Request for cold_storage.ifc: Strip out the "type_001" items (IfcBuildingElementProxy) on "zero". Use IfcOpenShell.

First a look at what the model holds.

```python
import ifcopenshell
import ifcopenshell.util.element

model = ifcopenshell.open("cold_storage.ifc")
print(model.schema)
storey = next(s for s in model.by_type("IfcBuildingStorey") if s.Name == "zero")
proxies = [e for e in ifcopenshell.util.element.get_decomposition(storey) if e.is_a("IfcBuildingElementProxy")]
seen = {}
for e in proxies:
    element_type = ifcopenshell.util.element.get_type(e)
    name = element_type.Name if element_type not in (None, e) else None
    seen[name] = seen.get(name, 0) + 1
for name, count in sorted(seen.items(), key=str):
    print(count, "x", name)
```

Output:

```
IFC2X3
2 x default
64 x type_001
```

```python
import ifcopenshell
import ifcopenshell.api.root
import ifcopenshell.util.element

model = ifcopenshell.open("cold_storage.ifc")

storey = next(s for s in model.by_type("IfcBuildingStorey") if s.Name == "zero")
proxies = [e for e in ifcopenshell.util.element.get_decomposition(storey) if e.is_a("IfcBuildingElementProxy")]
targets = [e for e in proxies if (t := ifcopenshell.util.element.get_type(e)) not in (None, e) and t.Name == "type_001"]

for e in targets:
    ifcopenshell.api.root.remove_product(model, product=e)
print(len(targets), "removed")

model.write("cold_storage_v2.ifc")
```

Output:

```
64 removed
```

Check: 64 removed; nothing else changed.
